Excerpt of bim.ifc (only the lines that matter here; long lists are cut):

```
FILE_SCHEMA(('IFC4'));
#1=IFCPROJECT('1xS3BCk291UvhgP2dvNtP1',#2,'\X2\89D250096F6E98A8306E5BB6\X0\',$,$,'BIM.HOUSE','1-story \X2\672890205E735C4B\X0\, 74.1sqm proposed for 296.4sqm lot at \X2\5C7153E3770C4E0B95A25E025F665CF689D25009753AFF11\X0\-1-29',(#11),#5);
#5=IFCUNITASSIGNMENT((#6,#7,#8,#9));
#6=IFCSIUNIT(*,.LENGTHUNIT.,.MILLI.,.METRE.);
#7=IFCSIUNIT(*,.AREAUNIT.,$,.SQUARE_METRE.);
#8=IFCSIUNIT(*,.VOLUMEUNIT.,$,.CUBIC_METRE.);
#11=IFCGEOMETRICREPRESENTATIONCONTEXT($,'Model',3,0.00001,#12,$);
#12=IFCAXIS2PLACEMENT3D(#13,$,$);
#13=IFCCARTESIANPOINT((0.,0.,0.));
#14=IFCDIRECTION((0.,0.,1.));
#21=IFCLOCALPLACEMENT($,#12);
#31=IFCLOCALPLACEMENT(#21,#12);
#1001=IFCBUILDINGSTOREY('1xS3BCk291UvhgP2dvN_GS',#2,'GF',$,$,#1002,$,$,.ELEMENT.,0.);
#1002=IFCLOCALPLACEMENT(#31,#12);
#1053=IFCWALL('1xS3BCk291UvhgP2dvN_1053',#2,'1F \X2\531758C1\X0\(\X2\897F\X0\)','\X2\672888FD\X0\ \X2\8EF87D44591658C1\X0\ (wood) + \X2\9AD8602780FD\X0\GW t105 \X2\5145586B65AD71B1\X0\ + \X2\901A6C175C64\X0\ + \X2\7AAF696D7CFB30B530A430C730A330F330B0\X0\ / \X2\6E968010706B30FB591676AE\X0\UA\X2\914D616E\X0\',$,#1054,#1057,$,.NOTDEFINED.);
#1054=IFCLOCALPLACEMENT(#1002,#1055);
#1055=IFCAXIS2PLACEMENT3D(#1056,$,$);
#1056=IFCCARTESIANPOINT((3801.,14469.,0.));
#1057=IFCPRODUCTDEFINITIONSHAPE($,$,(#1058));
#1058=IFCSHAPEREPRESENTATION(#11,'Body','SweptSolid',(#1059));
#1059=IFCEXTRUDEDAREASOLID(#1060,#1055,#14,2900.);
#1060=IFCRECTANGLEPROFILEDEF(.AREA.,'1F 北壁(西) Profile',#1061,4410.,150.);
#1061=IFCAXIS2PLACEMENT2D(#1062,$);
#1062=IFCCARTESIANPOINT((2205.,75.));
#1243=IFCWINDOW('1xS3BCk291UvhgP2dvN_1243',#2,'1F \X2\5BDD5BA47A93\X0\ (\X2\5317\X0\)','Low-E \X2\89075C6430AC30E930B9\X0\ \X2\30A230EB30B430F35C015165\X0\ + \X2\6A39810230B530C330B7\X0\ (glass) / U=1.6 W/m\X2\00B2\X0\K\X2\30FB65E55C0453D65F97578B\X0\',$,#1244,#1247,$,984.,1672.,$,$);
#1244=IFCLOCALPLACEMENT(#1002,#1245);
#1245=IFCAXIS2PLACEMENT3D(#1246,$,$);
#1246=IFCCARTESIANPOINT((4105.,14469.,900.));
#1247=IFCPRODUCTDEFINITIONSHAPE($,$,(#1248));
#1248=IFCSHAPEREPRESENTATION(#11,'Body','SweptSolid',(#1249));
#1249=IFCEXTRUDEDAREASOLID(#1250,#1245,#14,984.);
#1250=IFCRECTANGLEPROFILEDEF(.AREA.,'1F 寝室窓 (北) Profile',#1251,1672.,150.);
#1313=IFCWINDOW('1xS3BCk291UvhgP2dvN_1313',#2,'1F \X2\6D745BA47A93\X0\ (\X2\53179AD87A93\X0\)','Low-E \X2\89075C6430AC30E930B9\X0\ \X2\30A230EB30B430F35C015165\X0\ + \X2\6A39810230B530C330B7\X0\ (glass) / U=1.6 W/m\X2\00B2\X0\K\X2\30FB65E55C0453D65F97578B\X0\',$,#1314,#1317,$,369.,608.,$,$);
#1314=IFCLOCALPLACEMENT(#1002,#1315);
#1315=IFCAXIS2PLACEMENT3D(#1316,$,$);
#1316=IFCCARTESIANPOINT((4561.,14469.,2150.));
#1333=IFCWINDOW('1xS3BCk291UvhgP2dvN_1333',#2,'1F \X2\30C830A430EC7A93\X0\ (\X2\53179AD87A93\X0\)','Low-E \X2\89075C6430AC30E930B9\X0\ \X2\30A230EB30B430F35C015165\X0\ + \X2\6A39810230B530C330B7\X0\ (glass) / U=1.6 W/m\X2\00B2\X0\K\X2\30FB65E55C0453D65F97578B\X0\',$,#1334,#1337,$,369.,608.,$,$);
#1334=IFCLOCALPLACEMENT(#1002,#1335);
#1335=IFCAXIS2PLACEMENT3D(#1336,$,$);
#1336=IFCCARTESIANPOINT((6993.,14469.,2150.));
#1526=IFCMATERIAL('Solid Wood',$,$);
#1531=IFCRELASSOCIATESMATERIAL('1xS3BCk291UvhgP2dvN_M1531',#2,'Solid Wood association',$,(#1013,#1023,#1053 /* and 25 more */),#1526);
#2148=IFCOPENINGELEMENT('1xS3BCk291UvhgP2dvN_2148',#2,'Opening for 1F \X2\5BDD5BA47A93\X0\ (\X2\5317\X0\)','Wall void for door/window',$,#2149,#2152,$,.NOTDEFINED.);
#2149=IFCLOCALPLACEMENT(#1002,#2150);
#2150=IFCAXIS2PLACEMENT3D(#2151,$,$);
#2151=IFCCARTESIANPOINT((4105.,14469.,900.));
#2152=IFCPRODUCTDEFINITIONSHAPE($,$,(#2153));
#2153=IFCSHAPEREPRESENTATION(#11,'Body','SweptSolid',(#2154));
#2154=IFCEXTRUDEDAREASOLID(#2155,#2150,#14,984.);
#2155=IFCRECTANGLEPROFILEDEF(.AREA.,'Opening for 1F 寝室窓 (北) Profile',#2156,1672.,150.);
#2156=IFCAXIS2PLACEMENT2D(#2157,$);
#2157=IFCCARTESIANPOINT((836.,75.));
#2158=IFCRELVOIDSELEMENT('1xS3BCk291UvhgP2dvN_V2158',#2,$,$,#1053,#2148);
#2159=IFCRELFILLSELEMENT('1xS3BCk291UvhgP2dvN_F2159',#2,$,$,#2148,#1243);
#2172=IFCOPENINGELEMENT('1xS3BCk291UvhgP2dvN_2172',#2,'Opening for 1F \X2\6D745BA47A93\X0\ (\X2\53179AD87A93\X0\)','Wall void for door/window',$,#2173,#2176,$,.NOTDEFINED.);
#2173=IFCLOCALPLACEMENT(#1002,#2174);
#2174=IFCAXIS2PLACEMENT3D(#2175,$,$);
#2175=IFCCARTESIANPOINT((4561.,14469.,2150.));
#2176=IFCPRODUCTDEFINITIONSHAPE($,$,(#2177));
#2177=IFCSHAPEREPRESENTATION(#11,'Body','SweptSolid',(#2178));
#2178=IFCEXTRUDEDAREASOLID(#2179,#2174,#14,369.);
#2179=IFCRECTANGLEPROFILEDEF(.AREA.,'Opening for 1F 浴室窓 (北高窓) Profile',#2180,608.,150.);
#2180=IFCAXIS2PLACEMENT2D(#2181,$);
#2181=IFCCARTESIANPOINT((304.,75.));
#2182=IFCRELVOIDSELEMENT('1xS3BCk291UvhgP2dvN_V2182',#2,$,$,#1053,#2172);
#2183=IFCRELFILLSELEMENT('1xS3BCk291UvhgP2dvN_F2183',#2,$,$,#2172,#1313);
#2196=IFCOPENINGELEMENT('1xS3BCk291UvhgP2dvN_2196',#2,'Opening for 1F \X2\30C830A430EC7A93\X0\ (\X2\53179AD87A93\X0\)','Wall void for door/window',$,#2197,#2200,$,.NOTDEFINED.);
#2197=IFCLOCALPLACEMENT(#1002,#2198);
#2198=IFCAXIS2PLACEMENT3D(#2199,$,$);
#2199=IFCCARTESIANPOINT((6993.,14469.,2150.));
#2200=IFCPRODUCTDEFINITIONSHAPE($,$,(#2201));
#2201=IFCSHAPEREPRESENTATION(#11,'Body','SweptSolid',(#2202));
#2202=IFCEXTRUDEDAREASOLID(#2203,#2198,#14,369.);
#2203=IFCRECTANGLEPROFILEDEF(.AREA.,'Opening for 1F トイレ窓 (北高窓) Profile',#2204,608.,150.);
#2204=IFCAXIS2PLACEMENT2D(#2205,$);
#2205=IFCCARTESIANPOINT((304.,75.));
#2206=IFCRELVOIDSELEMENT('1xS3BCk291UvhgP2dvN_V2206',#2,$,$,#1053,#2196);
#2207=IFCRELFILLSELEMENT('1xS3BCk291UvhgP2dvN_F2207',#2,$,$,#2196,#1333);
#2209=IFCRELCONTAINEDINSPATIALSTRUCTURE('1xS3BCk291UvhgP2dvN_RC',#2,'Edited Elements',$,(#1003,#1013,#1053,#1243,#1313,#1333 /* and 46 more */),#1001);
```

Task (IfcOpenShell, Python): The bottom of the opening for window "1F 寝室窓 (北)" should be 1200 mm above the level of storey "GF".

```python
import numpy as np
import ifcopenshell
import ifcopenshell.api.geometry
import ifcopenshell.geom
import ifcopenshell.util.element
import ifcopenshell.util.placement
import ifcopenshell.util.shape
import ifcopenshell.util.unit

model = ifcopenshell.open("bim.ifc")
unit_scale = ifcopenshell.util.unit.calculate_unit_scale(model)

window = model.by_guid("1xS3BCk291UvhgP2dvN_1243")
opening = window.FillsVoids[0].RelatingOpeningElement
storey = ifcopenshell.util.element.get_container(window, ifc_class="IfcBuildingStorey")
level = ifcopenshell.util.placement.get_local_placement(storey.ObjectPlacement)[2, 3]

# The opening's origin need not be at the sill, so measure its lowest point.
shape = ifcopenshell.geom.create_shape(ifcopenshell.geom.settings(), opening)
bottom = ifcopenshell.util.shape.get_shape_bottom_elevation(shape, shape.geometry) / unit_scale
dz = level + 1200.0 - bottom

shift = np.array([0.0, 0.0, dz])
# The window is not placed relative to its opening, so move both.
for product in (opening, window):
    matrix = ifcopenshell.util.placement.get_local_placement(product.ObjectPlacement)
    matrix[:3, 3] += shift
    ifcopenshell.api.geometry.edit_object_placement(model, product=product, matrix=matrix, is_si=False)

print(f"moved by {dz * unit_scale:+.3f} m")

model.write("bim-out.ifc")
```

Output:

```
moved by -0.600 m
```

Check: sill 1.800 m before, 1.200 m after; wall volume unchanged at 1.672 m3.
